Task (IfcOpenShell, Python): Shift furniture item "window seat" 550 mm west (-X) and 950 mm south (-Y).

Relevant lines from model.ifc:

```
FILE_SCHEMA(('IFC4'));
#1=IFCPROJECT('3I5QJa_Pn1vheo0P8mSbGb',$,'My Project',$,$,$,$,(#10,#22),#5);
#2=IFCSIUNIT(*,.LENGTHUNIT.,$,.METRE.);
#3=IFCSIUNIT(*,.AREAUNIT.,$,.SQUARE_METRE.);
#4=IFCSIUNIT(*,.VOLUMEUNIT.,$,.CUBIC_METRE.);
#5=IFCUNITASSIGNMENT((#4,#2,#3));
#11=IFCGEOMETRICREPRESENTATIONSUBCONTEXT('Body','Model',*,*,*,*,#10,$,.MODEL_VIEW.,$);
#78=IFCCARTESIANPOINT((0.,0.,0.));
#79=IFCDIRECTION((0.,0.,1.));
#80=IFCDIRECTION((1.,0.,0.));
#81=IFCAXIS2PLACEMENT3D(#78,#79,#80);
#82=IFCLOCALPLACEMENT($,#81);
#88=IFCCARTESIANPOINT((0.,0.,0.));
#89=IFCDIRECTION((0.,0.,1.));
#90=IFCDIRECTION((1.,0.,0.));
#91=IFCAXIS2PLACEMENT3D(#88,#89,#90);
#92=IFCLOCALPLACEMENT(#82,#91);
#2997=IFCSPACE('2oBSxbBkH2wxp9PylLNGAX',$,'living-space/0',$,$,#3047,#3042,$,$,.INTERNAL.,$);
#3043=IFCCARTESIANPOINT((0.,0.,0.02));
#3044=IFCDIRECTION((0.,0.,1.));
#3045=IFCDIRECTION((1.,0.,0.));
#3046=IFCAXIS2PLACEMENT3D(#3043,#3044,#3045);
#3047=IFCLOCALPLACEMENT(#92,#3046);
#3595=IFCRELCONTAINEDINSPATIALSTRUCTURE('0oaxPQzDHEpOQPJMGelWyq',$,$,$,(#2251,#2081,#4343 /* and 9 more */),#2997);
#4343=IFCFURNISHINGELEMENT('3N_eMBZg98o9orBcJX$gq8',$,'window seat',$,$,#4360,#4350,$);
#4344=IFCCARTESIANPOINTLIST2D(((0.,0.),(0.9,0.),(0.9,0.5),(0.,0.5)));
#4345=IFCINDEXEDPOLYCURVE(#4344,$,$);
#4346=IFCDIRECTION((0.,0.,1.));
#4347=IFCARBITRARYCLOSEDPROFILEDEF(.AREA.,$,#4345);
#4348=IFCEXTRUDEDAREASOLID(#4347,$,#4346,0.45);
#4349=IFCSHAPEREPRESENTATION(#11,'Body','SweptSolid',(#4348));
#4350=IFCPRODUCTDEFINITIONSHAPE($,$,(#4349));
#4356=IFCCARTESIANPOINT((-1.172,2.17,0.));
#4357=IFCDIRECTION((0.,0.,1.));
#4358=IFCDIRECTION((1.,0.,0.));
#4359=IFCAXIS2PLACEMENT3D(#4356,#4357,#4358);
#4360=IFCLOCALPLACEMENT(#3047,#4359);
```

```python
import ifcopenshell
import ifcopenshell.api.geometry
import ifcopenshell.util.placement
import ifcopenshell.util.unit

model = ifcopenshell.open("model.ifc")
unit_scale = ifcopenshell.util.unit.calculate_unit_scale(model)

item = model.by_id(4343)
matrix = ifcopenshell.util.placement.get_local_placement(item.ObjectPlacement)
matrix[0, 3] -= 0.55 / unit_scale
matrix[1, 3] -= 0.95 / unit_scale
ifcopenshell.api.geometry.edit_object_placement(model, product=item, matrix=matrix, is_si=False)

print(ifcopenshell.util.placement.get_local_placement(item.ObjectPlacement).round(3) + 0.0)

model.write("model-out.ifc")
```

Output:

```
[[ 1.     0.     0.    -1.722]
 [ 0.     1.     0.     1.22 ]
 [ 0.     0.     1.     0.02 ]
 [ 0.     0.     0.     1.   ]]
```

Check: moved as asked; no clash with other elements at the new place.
